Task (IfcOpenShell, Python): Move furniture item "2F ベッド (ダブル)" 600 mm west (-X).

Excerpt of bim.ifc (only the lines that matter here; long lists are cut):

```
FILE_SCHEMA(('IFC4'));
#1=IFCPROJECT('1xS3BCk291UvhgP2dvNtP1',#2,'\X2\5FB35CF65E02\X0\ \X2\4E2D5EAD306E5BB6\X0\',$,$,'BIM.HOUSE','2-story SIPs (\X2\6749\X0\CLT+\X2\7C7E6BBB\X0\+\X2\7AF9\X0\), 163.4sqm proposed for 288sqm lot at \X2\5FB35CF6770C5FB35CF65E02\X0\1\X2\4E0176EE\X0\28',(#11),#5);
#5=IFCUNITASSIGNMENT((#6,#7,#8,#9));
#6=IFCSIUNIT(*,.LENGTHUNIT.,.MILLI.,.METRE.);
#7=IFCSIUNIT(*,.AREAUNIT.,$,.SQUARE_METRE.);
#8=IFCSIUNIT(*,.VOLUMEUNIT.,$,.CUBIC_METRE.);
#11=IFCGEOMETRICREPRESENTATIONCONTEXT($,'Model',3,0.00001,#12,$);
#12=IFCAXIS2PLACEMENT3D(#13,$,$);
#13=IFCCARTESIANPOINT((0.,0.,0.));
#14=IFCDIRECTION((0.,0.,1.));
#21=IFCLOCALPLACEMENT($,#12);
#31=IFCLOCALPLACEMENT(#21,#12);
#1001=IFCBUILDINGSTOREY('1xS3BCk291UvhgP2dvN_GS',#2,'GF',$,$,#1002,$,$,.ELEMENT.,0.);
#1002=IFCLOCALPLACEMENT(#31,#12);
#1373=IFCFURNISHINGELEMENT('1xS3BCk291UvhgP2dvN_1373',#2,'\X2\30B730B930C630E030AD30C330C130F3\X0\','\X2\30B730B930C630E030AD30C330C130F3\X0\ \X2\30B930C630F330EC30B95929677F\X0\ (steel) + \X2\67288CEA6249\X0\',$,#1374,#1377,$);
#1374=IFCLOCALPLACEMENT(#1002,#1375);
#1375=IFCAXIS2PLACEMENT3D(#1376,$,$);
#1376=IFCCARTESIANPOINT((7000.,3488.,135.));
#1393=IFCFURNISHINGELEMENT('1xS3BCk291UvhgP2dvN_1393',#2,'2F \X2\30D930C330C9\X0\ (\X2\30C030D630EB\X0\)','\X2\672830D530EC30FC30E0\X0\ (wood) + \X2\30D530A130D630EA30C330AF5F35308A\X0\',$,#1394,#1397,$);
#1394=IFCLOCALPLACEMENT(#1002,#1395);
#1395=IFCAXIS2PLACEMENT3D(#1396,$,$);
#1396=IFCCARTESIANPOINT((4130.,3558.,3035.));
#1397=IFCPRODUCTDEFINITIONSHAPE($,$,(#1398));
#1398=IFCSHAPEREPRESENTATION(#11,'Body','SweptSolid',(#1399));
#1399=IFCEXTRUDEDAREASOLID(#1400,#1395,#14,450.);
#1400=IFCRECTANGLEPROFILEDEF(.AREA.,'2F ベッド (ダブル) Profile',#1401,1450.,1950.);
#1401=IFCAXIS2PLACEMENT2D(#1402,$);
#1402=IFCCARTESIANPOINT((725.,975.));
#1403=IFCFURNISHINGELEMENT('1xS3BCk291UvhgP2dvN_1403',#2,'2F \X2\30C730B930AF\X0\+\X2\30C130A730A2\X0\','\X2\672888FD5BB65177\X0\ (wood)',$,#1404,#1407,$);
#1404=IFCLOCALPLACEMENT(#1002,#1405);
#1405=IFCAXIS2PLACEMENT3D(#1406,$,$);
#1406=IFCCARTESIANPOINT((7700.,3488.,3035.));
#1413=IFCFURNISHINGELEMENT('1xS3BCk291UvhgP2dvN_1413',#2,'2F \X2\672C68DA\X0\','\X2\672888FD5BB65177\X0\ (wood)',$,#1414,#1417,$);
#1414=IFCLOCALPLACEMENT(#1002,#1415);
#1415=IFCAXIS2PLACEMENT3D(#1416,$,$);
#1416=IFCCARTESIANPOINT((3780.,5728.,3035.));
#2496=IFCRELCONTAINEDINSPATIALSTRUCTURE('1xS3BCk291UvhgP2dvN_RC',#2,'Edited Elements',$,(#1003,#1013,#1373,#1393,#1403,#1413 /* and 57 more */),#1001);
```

```python
import ifcopenshell
import ifcopenshell.api.geometry
import ifcopenshell.util.placement
import ifcopenshell.util.unit

model = ifcopenshell.open("bim.ifc")
unit_scale = ifcopenshell.util.unit.calculate_unit_scale(model)

item = model.by_guid("1xS3BCk291UvhgP2dvN_1393")
matrix = ifcopenshell.util.placement.get_local_placement(item.ObjectPlacement)
matrix[0, 3] -= 0.6 / unit_scale
ifcopenshell.api.geometry.edit_object_placement(model, product=item, matrix=matrix, is_si=False)

print(ifcopenshell.util.placement.get_local_placement(item.ObjectPlacement).round(3) + 0.0)

model.write("bim_edited.ifc")
```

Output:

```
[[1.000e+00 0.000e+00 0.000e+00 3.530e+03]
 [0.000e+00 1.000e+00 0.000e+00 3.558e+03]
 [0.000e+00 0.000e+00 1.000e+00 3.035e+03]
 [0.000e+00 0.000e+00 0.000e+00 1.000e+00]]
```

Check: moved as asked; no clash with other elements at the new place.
